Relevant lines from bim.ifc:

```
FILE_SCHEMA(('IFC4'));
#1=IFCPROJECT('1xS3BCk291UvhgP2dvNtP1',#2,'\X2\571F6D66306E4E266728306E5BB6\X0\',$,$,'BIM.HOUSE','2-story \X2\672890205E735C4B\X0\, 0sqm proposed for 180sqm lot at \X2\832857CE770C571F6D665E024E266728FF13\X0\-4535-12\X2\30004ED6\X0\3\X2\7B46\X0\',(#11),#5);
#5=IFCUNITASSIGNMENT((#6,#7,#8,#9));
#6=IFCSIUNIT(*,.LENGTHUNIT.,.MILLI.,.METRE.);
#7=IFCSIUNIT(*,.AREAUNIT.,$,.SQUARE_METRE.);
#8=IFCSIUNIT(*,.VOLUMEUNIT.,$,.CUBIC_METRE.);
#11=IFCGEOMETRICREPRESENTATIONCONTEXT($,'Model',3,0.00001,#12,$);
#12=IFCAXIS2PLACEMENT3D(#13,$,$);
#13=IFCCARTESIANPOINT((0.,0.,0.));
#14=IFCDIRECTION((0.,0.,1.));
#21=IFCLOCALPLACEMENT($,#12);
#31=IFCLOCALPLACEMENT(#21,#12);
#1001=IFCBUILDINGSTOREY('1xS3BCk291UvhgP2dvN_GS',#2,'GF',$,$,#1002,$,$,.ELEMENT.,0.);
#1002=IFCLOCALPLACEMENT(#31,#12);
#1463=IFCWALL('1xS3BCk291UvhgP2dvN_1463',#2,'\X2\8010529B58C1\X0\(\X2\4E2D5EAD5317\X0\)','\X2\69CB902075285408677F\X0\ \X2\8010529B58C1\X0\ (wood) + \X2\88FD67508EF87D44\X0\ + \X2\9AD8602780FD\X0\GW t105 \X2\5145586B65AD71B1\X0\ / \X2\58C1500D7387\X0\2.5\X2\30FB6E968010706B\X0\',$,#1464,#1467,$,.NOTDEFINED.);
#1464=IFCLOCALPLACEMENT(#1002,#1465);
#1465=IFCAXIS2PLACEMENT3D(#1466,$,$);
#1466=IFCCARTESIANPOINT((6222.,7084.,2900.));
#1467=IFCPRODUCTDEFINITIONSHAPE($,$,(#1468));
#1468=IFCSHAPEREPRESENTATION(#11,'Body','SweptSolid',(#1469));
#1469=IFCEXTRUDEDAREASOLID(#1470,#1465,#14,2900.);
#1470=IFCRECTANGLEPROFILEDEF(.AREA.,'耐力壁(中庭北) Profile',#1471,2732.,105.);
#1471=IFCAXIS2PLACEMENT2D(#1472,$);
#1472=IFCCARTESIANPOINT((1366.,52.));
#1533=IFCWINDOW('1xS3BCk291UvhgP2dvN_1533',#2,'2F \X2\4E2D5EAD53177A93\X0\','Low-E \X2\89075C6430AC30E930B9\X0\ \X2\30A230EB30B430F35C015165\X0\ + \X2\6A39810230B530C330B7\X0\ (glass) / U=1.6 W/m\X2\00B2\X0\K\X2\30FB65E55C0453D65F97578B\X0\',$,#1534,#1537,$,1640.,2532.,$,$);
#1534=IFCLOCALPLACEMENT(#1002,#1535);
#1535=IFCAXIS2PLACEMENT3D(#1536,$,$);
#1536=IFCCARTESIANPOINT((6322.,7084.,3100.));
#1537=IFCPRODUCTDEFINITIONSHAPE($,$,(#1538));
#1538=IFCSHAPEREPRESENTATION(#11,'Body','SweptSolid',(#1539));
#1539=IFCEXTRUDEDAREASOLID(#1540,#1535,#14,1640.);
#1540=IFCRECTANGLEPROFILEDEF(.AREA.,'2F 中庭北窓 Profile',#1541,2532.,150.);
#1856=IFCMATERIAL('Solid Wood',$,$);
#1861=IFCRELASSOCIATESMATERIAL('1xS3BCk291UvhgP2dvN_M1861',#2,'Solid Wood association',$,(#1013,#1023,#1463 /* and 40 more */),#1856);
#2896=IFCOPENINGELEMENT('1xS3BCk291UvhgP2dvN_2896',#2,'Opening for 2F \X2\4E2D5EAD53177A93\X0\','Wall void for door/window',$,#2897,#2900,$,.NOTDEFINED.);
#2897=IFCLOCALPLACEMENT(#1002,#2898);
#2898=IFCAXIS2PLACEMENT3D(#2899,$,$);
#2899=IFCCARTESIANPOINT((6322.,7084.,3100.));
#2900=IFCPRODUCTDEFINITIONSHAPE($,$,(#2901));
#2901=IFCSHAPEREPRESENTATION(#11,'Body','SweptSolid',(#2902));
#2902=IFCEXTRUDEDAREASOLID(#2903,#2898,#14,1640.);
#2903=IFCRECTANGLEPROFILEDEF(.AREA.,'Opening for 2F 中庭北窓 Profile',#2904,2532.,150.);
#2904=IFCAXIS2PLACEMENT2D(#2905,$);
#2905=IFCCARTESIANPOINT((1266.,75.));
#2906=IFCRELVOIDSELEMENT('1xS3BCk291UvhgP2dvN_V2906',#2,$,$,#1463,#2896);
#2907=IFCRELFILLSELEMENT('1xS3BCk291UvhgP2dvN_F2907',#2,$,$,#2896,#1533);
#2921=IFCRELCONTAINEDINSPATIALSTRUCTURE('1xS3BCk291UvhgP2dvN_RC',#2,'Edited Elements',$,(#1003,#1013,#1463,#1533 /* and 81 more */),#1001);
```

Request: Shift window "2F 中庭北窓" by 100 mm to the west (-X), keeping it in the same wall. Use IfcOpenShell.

```python
import ifcopenshell
import ifcopenshell.api.geometry
import ifcopenshell.util.placement
import ifcopenshell.util.unit

model = ifcopenshell.open("bim.ifc")
unit_scale = ifcopenshell.util.unit.calculate_unit_scale(model)

window = model.by_guid("1xS3BCk291UvhgP2dvN_1533")
opening = window.FillsVoids[0].RelatingOpeningElement
wall = opening.VoidsElements[0].RelatingBuildingElement

wall_matrix = ifcopenshell.util.placement.get_local_placement(wall.ObjectPlacement)
shift = wall_matrix[:3, 0] * -0.1 / unit_scale
before = ifcopenshell.util.placement.get_local_placement(window.ObjectPlacement)[:3, 3].copy()

# The window is not placed relative to its opening, so move both.
for product in (opening, window):
    matrix = ifcopenshell.util.placement.get_local_placement(product.ObjectPlacement)
    matrix[:3, 3] += shift
    ifcopenshell.api.geometry.edit_object_placement(model, product=product, matrix=matrix, is_si=False)

after = ifcopenshell.util.placement.get_local_placement(window.ObjectPlacement)[:3, 3]
print("window moved by", (after - before).round(3) + 0.0)

model.write("bim_edited.ifc")
```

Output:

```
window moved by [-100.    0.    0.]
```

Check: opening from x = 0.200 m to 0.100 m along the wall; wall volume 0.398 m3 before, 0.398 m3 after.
